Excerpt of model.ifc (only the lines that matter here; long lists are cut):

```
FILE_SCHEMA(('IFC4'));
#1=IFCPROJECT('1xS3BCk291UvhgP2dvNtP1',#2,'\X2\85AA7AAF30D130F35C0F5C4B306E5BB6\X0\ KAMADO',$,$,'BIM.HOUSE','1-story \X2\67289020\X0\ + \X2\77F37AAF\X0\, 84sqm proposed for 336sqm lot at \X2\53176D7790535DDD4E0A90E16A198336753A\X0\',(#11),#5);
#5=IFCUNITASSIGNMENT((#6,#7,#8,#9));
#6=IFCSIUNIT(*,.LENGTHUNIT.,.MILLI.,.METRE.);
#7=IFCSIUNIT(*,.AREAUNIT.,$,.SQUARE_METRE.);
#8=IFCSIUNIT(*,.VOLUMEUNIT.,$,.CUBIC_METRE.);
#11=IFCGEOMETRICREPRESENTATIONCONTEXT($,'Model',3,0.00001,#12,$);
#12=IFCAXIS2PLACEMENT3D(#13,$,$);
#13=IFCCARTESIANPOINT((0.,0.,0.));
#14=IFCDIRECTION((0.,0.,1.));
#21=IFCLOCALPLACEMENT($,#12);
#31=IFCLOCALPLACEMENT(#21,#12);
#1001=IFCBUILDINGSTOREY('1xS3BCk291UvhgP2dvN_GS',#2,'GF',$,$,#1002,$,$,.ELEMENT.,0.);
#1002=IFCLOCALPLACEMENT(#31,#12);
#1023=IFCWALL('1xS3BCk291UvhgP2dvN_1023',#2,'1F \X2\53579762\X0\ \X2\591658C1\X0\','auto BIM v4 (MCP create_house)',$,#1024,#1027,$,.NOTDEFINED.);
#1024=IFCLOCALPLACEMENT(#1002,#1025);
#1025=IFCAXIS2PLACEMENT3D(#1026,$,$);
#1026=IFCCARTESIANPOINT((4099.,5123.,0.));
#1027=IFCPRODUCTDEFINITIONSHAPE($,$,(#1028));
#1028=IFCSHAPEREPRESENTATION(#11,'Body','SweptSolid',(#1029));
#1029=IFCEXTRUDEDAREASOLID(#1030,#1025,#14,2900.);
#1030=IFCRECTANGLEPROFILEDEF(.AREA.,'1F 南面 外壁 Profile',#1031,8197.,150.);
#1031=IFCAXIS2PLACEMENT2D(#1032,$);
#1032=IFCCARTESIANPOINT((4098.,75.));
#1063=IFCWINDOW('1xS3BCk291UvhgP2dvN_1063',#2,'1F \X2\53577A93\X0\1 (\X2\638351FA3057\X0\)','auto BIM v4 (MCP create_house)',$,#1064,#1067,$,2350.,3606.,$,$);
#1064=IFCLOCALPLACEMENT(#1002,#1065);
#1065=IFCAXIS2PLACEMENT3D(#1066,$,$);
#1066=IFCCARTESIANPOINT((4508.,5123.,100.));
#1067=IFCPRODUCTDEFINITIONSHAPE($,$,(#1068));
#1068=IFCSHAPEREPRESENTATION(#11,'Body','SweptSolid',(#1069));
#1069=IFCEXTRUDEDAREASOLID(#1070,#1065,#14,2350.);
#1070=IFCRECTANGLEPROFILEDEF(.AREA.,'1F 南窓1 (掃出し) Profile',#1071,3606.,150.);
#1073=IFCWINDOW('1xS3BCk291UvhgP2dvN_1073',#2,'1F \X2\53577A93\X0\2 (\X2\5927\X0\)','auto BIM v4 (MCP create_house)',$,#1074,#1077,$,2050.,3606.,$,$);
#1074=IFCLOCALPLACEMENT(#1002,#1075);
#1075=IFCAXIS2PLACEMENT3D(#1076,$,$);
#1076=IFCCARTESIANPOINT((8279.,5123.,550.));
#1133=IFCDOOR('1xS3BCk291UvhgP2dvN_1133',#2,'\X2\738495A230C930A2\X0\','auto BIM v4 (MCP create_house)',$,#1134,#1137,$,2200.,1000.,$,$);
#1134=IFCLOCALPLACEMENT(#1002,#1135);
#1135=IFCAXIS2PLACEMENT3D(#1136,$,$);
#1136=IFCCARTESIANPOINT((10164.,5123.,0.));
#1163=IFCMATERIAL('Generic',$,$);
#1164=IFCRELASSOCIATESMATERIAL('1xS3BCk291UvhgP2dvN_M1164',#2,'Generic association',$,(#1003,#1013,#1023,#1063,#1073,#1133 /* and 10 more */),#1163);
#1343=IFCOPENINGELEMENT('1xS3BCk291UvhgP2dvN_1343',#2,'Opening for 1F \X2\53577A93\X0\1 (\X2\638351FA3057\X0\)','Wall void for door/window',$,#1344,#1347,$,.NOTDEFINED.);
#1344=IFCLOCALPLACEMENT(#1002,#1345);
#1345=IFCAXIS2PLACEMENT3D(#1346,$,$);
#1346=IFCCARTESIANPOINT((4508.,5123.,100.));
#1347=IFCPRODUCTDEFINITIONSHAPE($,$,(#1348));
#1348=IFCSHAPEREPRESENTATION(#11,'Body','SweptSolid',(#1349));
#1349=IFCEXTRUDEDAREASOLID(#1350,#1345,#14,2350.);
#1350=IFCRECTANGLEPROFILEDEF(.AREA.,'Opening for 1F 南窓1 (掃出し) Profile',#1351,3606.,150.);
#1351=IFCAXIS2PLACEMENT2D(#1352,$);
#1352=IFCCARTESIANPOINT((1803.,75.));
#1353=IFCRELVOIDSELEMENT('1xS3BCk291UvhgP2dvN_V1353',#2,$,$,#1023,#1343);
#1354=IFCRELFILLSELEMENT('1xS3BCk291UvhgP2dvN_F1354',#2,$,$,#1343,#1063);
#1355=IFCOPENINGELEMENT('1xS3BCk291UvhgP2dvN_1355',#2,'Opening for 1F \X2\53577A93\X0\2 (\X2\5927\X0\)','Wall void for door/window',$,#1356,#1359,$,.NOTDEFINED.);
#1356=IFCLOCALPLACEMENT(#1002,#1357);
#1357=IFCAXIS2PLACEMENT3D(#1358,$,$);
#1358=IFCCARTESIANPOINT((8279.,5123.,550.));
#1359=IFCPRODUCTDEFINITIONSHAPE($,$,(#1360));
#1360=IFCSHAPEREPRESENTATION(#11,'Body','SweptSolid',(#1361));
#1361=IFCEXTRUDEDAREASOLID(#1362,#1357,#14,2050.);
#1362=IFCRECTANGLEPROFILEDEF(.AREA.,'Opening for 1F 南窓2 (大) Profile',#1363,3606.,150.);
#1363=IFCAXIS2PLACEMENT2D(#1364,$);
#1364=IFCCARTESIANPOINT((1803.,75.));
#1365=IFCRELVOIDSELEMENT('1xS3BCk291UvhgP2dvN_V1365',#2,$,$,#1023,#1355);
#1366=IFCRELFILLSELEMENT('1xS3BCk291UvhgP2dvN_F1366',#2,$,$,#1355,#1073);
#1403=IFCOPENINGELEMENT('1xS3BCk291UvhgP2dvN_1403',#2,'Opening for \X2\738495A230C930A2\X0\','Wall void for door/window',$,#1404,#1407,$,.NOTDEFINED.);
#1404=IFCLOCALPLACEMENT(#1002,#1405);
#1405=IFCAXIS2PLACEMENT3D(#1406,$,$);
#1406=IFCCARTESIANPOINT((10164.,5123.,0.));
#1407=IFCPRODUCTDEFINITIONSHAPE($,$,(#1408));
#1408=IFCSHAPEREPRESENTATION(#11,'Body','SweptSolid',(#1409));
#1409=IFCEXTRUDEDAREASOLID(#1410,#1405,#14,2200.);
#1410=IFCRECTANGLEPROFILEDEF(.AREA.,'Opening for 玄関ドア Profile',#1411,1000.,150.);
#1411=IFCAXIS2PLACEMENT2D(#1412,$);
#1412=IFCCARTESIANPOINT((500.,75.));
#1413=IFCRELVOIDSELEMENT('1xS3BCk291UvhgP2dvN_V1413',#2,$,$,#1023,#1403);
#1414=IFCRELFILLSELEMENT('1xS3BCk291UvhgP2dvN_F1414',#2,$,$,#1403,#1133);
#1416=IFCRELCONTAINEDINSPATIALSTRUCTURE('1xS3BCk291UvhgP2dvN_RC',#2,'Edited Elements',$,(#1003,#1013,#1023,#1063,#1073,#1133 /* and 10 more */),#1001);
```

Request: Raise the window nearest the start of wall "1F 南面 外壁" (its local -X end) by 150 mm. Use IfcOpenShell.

```python
import numpy as np
import ifcopenshell
import ifcopenshell.api.geometry
import ifcopenshell.util.placement
import ifcopenshell.util.unit

model = ifcopenshell.open("model.ifc")
unit_scale = ifcopenshell.util.unit.calculate_unit_scale(model)

window = model.by_guid("1xS3BCk291UvhgP2dvN_1063")
opening = window.FillsVoids[0].RelatingOpeningElement
dz = 150.0

shift = np.array([0.0, 0.0, dz])
# The window is not placed relative to its opening, so move both.
for product in (opening, window):
    matrix = ifcopenshell.util.placement.get_local_placement(product.ObjectPlacement)
    matrix[:3, 3] += shift
    ifcopenshell.api.geometry.edit_object_placement(model, product=product, matrix=matrix, is_si=False)

print(f"moved by {dz * unit_scale:+.3f} m")

model.write("model_updated.ifc")
```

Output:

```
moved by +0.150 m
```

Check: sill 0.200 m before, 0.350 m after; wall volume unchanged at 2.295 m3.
